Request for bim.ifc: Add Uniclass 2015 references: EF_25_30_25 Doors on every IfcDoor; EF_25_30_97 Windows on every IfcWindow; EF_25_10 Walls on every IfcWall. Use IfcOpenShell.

First a look at what the model holds.

```python
import ifcopenshell

model = ifcopenshell.open("bim.ifc")
print(model.schema)
print("classifications:", [c.Name for c in model.by_type("IfcClassification")])
for ifc_class in ("IfcDoor", "IfcRoof", "IfcStair", "IfcWall", "IfcWindow"):
    print(ifc_class, len(model.by_type(ifc_class)))
```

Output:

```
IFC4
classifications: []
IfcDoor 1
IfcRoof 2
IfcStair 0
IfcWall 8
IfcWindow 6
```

```python
import ifcopenshell
import ifcopenshell.api.classification

model = ifcopenshell.open("bim.ifc")

system = ifcopenshell.api.classification.add_classification(model, classification="Uniclass 2015")

codes = {
    "IfcDoor": ("EF_25_30_25", "Doors"),
    "IfcWindow": ("EF_25_30_97", "Windows"),
    "IfcWall": ("EF_25_10", "Walls"),
}
for ifc_class, (code, name) in codes.items():
    products = model.by_type(ifc_class)
    ifcopenshell.api.classification.add_reference(
        model, products=products, classification=system, identification=code, name=name
    )
    print(code, len(products))

model.write("bim-out.ifc")
```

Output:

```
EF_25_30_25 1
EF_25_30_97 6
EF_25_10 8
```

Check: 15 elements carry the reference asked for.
